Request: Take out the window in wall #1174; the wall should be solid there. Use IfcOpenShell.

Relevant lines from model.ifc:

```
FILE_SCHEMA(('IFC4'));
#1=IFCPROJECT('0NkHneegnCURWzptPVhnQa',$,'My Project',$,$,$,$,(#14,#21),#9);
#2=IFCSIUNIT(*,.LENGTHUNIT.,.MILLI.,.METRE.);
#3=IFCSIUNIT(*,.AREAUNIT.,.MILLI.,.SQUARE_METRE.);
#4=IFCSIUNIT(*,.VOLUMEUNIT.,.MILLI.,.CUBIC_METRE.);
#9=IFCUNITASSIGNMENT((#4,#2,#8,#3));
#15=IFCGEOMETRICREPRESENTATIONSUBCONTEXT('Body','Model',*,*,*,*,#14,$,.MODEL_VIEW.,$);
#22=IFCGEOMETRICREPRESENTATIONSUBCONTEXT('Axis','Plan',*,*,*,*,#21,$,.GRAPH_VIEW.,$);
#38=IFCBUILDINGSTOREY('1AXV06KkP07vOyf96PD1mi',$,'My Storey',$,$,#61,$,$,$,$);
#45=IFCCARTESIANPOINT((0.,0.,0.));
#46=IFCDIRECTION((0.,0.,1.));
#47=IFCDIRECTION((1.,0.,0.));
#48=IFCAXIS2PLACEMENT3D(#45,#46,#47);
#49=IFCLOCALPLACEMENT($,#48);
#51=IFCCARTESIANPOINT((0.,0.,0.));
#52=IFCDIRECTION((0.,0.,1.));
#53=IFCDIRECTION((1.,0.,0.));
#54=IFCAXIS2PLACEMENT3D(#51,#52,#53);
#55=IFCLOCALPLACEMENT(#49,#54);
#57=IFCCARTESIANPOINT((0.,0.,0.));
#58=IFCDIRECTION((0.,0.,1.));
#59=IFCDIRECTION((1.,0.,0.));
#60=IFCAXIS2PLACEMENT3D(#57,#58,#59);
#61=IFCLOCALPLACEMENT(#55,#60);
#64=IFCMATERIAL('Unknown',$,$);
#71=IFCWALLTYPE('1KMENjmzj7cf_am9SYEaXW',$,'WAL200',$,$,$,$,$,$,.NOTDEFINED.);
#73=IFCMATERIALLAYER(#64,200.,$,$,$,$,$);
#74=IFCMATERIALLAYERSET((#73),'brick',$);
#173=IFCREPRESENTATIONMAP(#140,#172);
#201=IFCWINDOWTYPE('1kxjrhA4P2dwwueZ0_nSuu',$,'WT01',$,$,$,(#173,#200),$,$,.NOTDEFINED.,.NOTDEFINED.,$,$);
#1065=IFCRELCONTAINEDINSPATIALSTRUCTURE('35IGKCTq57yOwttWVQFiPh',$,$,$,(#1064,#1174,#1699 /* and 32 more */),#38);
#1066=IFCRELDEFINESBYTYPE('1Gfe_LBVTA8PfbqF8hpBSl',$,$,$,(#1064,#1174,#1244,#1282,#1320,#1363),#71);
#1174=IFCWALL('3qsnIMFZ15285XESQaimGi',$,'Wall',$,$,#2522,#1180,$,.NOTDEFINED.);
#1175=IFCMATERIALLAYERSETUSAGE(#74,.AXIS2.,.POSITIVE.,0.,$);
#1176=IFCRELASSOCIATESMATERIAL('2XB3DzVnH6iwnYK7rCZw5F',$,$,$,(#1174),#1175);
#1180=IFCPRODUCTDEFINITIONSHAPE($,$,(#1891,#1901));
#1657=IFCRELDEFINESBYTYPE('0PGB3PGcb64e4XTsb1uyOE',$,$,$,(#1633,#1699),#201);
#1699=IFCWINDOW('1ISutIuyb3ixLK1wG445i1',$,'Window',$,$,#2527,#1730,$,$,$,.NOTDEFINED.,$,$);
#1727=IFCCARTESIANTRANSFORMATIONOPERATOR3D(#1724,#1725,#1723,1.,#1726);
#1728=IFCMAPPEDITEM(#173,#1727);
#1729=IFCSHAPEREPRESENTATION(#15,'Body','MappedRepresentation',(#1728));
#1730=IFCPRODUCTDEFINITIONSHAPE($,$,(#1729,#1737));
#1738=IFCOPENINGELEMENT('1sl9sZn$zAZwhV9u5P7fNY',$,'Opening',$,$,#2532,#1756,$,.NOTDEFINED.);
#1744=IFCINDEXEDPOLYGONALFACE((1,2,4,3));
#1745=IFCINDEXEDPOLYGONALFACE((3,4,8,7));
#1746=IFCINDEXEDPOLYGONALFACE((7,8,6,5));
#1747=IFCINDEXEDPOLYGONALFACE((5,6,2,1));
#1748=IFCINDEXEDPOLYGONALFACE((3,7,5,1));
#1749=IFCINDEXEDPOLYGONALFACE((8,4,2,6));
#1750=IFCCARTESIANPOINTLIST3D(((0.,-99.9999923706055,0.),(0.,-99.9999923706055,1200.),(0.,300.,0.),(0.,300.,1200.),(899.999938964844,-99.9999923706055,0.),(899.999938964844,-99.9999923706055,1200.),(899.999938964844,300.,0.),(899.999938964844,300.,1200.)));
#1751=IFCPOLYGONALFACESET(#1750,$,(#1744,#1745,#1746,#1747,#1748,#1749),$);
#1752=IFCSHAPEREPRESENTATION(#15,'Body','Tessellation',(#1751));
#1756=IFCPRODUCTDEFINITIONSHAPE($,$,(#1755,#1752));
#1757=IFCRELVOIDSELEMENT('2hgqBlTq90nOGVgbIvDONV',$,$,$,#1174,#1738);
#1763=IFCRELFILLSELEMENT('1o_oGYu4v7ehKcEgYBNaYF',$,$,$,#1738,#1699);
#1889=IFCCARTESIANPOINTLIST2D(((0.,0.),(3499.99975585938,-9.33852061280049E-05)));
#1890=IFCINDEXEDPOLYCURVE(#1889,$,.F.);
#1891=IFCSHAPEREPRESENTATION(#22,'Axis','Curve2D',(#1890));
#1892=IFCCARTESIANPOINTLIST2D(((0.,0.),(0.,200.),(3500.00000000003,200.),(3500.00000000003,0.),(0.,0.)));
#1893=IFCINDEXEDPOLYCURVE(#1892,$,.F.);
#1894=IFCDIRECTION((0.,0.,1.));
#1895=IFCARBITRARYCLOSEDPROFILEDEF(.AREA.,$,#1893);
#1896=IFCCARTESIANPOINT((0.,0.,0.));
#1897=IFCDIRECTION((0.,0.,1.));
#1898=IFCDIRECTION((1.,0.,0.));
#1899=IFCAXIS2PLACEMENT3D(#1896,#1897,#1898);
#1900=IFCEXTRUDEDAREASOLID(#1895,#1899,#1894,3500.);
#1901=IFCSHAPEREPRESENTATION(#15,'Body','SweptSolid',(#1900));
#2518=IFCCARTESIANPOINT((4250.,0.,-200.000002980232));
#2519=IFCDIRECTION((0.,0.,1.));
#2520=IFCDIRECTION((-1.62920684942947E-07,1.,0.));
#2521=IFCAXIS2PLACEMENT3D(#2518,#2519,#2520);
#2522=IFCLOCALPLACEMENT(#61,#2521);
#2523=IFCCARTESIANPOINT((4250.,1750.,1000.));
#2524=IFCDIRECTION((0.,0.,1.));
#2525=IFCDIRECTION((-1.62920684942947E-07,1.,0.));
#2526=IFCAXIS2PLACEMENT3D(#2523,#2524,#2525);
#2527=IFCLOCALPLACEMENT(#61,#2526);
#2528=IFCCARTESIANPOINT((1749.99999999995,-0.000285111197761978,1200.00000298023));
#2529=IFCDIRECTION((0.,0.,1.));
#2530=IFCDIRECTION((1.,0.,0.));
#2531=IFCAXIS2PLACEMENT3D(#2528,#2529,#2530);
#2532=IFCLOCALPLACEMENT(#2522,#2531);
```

```python
import ifcopenshell
import ifcopenshell.api.feature
import ifcopenshell.api.root
import ifcopenshell.geom
import ifcopenshell.util.shape

model = ifcopenshell.open("model.ifc")
settings = ifcopenshell.geom.settings()


def volume(element):
    """Net volume in cubic metres, openings subtracted."""
    shape = ifcopenshell.geom.create_shape(settings, element)
    return ifcopenshell.util.shape.get_volume(shape.geometry)


window = model.by_id(1699)
opening = window.FillsVoids[0].RelatingOpeningElement
wall = opening.VoidsElements[0].RelatingBuildingElement
before = volume(wall)

ifcopenshell.api.root.remove_product(model, product=window)
ifcopenshell.api.feature.remove_feature(model, feature=opening)

after = volume(wall)

print(f"wall volume {before:.3f} -> {after:.3f} m3")

model.write("model_edited.ifc")
```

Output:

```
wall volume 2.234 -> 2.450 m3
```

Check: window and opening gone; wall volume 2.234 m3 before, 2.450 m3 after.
